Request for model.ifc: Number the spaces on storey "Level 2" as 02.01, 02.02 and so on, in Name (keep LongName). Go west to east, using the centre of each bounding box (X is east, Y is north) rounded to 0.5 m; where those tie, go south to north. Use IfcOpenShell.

First a look at what the model holds.

```python
import ifcopenshell
import ifcopenshell.util.element
import ifcopenshell.util.placement

model = ifcopenshell.open("model.ifc")
print(model.schema)
storey = next(s for s in model.by_type("IfcBuildingStorey") if s.Name == "Level 2")
spaces = [e for e in ifcopenshell.util.element.get_decomposition(storey) if e.is_a("IfcSpace")]
for e in sorted(spaces, key=lambda e: e.id()):
    origin = ifcopenshell.util.placement.get_local_placement(e.ObjectPlacement)[:3, 3]
    print(e.id(), e.Name, e.LongName, origin.round(2) + 0.0, sep=" | ")
```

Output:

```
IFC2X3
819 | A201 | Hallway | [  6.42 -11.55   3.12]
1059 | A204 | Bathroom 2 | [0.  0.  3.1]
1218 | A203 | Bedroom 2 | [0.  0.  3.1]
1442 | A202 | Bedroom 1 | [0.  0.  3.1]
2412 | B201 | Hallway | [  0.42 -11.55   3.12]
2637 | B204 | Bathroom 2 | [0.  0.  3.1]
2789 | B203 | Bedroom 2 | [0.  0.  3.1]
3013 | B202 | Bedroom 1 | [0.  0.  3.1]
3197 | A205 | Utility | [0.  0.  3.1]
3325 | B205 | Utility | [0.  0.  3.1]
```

```python
import ifcopenshell
import ifcopenshell.geom
import ifcopenshell.util.element
import ifcopenshell.util.shape

model = ifcopenshell.open("model.ifc")
settings = ifcopenshell.geom.settings()
settings.set("use-world-coords", True)


def centre(element):
    shape = ifcopenshell.geom.create_shape(settings, element)
    return ifcopenshell.util.shape.get_bbox_centroid(shape.geometry)


storey = next(s for s in model.by_type("IfcBuildingStorey") if s.Name == "Level 2")
spaces = [e for e in ifcopenshell.util.element.get_decomposition(storey) if e.is_a("IfcSpace")]

# Insertion points can sit at a corner or the storey origin, so sort by the geometry (in metres).
centres = {e: centre(e) for e in spaces}
spaces.sort(key=lambda e: (round(centres[e][0] / 0.5), centres[e][1]))

for i, e in enumerate(spaces, start=1):
    number = f"02.{i:02d}"
    e.Name = number
    print(e.id(), number)

model.write("model_v2.ifc")
```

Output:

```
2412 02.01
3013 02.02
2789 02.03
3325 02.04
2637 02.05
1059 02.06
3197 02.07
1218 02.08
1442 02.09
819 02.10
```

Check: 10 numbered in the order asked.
